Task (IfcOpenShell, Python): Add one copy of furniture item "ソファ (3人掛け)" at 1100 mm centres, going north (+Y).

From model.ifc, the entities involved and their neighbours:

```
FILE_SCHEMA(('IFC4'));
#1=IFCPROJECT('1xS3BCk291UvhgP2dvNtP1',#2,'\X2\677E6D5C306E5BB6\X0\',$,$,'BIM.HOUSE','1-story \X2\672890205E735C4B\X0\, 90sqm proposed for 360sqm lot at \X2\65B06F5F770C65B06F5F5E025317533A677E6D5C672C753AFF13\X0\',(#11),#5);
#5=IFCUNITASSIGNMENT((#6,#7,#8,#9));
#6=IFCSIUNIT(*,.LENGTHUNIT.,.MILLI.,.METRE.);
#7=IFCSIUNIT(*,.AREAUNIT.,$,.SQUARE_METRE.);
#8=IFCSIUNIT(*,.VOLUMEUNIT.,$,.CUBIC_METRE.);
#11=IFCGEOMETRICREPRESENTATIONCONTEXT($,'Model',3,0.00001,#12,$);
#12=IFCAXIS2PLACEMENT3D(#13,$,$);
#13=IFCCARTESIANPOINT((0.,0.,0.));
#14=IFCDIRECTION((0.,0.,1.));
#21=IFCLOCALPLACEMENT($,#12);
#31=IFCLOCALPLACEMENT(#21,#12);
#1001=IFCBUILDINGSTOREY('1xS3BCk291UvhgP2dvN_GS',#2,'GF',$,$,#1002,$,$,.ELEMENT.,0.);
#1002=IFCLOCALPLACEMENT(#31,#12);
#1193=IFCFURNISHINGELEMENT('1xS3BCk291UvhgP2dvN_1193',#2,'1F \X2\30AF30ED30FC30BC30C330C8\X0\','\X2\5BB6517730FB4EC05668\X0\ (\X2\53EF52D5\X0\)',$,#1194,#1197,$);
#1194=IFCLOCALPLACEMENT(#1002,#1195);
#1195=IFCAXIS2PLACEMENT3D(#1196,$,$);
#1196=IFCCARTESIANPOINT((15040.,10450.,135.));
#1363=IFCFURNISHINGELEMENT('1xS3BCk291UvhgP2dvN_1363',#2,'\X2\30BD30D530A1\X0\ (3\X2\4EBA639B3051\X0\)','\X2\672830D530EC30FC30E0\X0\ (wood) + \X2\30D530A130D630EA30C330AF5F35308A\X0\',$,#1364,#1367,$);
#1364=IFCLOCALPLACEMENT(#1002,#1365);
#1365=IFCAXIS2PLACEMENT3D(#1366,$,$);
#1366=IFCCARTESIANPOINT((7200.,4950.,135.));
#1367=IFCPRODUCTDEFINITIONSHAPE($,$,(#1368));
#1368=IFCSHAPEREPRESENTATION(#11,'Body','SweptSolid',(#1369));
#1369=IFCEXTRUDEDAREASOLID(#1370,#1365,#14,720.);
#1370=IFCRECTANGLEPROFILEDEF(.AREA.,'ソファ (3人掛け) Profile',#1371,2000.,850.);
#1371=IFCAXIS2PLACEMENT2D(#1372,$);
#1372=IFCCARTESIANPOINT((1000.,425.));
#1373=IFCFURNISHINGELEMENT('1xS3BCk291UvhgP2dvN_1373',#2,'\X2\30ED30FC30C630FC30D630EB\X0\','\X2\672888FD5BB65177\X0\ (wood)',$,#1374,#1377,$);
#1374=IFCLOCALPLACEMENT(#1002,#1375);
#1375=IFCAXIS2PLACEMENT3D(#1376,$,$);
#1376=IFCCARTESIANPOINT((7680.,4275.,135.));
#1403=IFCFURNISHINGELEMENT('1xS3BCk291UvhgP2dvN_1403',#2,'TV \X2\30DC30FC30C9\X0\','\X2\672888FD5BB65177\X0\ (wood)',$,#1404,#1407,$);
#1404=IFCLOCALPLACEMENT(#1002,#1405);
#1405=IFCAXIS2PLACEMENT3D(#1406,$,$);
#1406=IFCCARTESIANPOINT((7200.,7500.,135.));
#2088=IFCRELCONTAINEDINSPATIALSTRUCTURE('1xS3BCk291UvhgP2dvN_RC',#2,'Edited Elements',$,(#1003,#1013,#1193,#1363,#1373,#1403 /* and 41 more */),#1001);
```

```python
import numpy as np
import ifcopenshell
import ifcopenshell.api.geometry
import ifcopenshell.api.root
import ifcopenshell.util.element
import ifcopenshell.util.placement

model = ifcopenshell.open("model.ifc")


def reuse_history(source, copy):
    """copy_class also copies each property set's owner history, people and application; keep the originals."""
    for rel in copy.IsDefinedBy:
        if rel.is_a("IfcRelDefinesByProperties") and (history := rel.RelatingPropertyDefinition.OwnerHistory):
            rel.RelatingPropertyDefinition.OwnerHistory = source.OwnerHistory
            ifcopenshell.util.element.remove_deep2(model, history)


source = model.by_guid("1xS3BCk291UvhgP2dvN_1363")
base = ifcopenshell.util.placement.get_local_placement(source.ObjectPlacement)
step = np.array([0.0, 1.0, 0.0]) * 1100.0

for i in range(1, 2):
    copy = ifcopenshell.api.root.copy_class(model, product=source)
    copy.Representation = ifcopenshell.util.element.copy_deep(
        model, source.Representation, exclude=["IfcGeometricRepresentationContext", "IfcRepresentationMap"]
    )
    reuse_history(source, copy)
    matrix = base.copy()
    matrix[:3, 3] += i * step
    print("added at", matrix[:3, 3].round(3) + 0.0)
    ifcopenshell.api.geometry.edit_object_placement(model, product=copy, matrix=matrix, is_si=False)

model.write("model_updated.ifc")
```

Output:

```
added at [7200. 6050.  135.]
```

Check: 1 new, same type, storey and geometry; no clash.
